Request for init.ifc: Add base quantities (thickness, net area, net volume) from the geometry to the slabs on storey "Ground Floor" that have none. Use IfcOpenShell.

First a look at what the model holds.

```python
import ifcopenshell
import ifcopenshell.util.element
import ifcopenshell.util.unit

model = ifcopenshell.open("init.ifc")
print(model.schema)
for unit_type in ("LENGTHUNIT", "AREAUNIT", "VOLUMEUNIT"):
    print(unit_type, ifcopenshell.util.unit.calculate_unit_scale(model, unit_type))
storey = next(s for s in model.by_type("IfcBuildingStorey") if s.Name == "Ground Floor")
slabs = [e for e in ifcopenshell.util.element.get_decomposition(storey) if e.is_a("IfcSlab")]
for e in sorted(slabs, key=lambda e: e.id()):
    print(e.id(), e.is_a(), e.Name, list(ifcopenshell.util.element.get_psets(e, qtos_only=True)), sep=" | ")
```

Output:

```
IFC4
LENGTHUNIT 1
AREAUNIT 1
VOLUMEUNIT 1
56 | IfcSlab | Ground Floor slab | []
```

```python
import ifcopenshell
import ifcopenshell.api.pset
import ifcopenshell.geom
import ifcopenshell.util.element
import ifcopenshell.util.shape
import ifcopenshell.util.unit

model = ifcopenshell.open("init.ifc")
unit_scale = ifcopenshell.util.unit.calculate_unit_scale(model)
area_scale = ifcopenshell.util.unit.calculate_unit_scale(model, "AREAUNIT")
volume_scale = ifcopenshell.util.unit.calculate_unit_scale(model, "VOLUMEUNIT")
settings = ifcopenshell.geom.settings()

storey = next(s for s in model.by_type("IfcBuildingStorey") if s.Name == "Ground Floor")
slabs = [e for e in ifcopenshell.util.element.get_decomposition(storey) if e.is_a("IfcSlab")]

for e in sorted(slabs, key=lambda e: e.id()):
    if ifcopenshell.util.element.get_psets(e, qtos_only=True, should_inherit=False):
        continue
    # Geometry comes back in metres, in the element's own axes.
    shape = ifcopenshell.geom.create_shape(settings, e)
    values = {
        "Width": ifcopenshell.util.shape.get_z(shape.geometry) / unit_scale,
        "NetArea": ifcopenshell.util.shape.get_footprint_area(shape.geometry) / area_scale,
        "NetVolume": ifcopenshell.util.shape.get_volume(shape.geometry) / volume_scale,
    }
    qto = ifcopenshell.api.pset.add_qto(model, product=e, name="Qto_SlabBaseQuantities")
    ifcopenshell.api.pset.edit_qto(model, qto=qto, properties=values)
    print(e.id(), {k: round(v, 3) for k, v in values.items()})

model.write("init_edited.ifc")
```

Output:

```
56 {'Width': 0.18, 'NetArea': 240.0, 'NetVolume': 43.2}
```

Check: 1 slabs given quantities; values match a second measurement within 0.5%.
